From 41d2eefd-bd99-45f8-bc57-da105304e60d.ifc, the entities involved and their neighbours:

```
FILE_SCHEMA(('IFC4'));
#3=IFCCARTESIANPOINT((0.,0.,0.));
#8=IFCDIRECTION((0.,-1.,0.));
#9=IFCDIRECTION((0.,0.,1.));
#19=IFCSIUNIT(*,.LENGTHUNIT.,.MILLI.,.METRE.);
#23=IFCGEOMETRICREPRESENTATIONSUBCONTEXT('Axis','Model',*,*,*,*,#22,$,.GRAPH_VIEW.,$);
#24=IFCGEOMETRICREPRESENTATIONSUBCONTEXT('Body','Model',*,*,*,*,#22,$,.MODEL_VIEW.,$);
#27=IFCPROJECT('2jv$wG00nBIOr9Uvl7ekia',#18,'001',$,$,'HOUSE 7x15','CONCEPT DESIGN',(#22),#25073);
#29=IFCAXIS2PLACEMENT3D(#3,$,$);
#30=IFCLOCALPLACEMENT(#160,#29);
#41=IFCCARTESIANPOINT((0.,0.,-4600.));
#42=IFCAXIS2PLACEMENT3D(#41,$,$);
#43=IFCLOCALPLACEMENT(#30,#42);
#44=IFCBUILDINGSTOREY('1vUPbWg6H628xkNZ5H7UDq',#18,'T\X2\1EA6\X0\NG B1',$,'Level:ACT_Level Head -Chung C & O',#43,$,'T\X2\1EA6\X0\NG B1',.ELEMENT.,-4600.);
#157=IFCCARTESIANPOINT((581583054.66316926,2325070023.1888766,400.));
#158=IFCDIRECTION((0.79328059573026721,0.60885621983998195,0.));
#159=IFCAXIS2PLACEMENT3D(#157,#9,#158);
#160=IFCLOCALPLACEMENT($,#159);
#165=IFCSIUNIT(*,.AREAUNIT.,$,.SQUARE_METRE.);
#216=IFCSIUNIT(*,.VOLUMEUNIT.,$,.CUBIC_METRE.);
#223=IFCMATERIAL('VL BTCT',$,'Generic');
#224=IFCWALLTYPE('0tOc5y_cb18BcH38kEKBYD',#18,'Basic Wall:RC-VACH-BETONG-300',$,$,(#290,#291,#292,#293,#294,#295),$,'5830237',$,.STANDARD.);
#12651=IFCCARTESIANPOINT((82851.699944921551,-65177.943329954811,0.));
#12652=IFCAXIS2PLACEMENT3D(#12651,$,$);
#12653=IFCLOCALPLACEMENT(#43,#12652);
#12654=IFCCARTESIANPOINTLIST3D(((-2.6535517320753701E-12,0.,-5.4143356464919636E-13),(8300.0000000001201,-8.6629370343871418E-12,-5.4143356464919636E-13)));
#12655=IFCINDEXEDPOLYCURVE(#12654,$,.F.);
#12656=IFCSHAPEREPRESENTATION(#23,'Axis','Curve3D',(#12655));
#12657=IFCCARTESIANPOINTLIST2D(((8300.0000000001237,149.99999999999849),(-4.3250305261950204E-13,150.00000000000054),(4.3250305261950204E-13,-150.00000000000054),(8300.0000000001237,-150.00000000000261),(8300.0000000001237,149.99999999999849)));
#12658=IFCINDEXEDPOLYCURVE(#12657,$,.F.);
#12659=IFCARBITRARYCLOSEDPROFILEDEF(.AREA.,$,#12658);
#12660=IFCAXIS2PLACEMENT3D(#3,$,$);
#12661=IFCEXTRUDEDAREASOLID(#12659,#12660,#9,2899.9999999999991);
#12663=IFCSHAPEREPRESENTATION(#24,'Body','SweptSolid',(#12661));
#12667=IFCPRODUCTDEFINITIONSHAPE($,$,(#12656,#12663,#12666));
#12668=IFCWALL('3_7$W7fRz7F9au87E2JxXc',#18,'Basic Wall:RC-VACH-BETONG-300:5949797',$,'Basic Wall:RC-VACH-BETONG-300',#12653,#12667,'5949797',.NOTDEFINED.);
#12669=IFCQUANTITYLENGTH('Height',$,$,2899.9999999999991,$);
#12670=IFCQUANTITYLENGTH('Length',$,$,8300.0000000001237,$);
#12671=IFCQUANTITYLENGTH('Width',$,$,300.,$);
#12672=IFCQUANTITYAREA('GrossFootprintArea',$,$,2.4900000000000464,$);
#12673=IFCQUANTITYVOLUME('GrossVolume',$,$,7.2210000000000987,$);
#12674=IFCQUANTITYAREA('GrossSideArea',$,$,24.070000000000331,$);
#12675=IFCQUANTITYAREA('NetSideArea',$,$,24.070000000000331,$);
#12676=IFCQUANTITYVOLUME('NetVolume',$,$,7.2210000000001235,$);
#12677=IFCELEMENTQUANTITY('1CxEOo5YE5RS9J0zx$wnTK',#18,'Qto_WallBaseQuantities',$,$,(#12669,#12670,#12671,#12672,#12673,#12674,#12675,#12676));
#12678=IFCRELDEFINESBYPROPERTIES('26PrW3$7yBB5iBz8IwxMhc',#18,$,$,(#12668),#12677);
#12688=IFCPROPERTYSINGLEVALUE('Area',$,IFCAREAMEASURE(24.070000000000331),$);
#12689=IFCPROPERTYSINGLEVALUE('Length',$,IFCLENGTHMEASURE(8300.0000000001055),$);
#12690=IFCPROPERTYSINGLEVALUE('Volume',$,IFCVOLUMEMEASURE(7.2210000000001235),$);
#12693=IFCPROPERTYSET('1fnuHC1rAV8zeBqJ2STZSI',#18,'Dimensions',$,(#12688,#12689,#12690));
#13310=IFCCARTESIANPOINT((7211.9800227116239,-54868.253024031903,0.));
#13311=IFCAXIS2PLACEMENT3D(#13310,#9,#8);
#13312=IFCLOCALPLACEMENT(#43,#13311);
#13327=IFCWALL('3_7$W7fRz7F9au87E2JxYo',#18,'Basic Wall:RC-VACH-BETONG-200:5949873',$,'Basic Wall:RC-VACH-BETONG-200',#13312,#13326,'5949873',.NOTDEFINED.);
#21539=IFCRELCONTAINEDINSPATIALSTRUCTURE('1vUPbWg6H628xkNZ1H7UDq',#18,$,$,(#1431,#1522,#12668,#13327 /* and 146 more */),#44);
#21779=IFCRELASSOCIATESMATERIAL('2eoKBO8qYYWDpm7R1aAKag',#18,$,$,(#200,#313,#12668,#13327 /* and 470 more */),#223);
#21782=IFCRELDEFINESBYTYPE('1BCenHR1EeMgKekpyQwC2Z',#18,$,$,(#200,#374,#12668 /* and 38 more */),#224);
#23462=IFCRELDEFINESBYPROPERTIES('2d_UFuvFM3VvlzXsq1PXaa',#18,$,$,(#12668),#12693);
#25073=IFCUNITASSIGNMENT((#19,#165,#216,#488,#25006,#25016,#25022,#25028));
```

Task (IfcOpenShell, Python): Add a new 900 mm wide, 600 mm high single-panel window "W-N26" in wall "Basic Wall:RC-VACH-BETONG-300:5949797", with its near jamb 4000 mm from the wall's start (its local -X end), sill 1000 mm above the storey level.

```python
import numpy as np
import ifcopenshell
import ifcopenshell.api.feature
import ifcopenshell.api.geometry
import ifcopenshell.api.pset
import ifcopenshell.api.root
import ifcopenshell.api.spatial
import ifcopenshell.geom
import ifcopenshell.util.element
import ifcopenshell.util.placement
import ifcopenshell.util.representation
import ifcopenshell.util.shape
import ifcopenshell.util.unit

model = ifcopenshell.open("41d2eefd-bd99-45f8-bc57-da105304e60d.ifc")
unit_scale = ifcopenshell.util.unit.calculate_unit_scale(model)
area_scale = ifcopenshell.util.unit.calculate_unit_scale(model, "AREAUNIT")
volume_scale = ifcopenshell.util.unit.calculate_unit_scale(model, "VOLUMEUNIT")
settings = ifcopenshell.geom.settings()


def volume(element):
    """Net volume in cubic metres, openings subtracted."""
    shape = ifcopenshell.geom.create_shape(settings, element)
    return ifcopenshell.util.shape.get_volume(shape.geometry)


wall = model.by_guid("3_7$W7fRz7F9au87E2JxXc")
storey = ifcopenshell.util.element.get_container(wall, ifc_class="IfcBuildingStorey")
context = ifcopenshell.util.representation.get_context(model, "Model", "Body", "MODEL_VIEW")
before = volume(wall)

width, height, from_end, sill = 0.9, 0.6, 4, 1  # metres

# The wall runs along its own X axis, and the end named is its -X end.
wall_shape = ifcopenshell.geom.create_shape(settings, wall)
x, y, z = ifcopenshell.util.shape.get_vertices(wall_shape.geometry).T
start = x.min() + from_end
face, thickness = float(y.min()), float(y.max() - y.min())
wall_matrix = ifcopenshell.util.placement.get_local_placement(wall.ObjectPlacement)
level = ifcopenshell.util.placement.get_local_placement(storey.ObjectPlacement)[2, 3]


def in_wall(x, y):
    """Placement at x, y metres in the wall's axes, at sill height."""
    matrix = wall_matrix.copy()
    matrix[:, 3] = wall_matrix @ np.array([x / unit_scale, y / unit_scale, 0.0, 1.0])
    matrix[2, 3] = level + sill / unit_scale
    return matrix


# Opening: a box that overshoots both wall faces by 50 mm.
opening = ifcopenshell.api.root.create_entity(model, ifc_class="IfcOpeningElement", predefined_type="OPENING")
box = ifcopenshell.api.geometry.add_wall_representation(
    model, context=context, length=width, height=height, thickness=thickness + 0.1
)
ifcopenshell.api.geometry.assign_representation(model, product=opening, representation=box)
ifcopenshell.api.geometry.edit_object_placement(model, product=opening, matrix=in_wall(start, face - 0.05), is_si=False)
ifcopenshell.api.feature.add_feature(model, feature=opening, element=wall)

window = ifcopenshell.api.root.create_entity(model, ifc_class="IfcWindow", name="W-N26", predefined_type="WINDOW")
window.OverallWidth, window.OverallHeight = width / unit_scale, height / unit_scale
window.PartitioningType = "SINGLE_PANEL"
body = ifcopenshell.api.geometry.add_window_representation(
    model,
    context=context,
    overall_width=window.OverallWidth,
    overall_height=window.OverallHeight,
    partition_type="SINGLE_PANEL",
)
ifcopenshell.api.geometry.assign_representation(model, product=window, representation=body)
ifcopenshell.api.spatial.assign_container(model, products=[window], relating_structure=storey)
ifcopenshell.api.feature.add_filling(model, opening=opening, element=window)

# Centre the window in the wall's thickness.
ifcopenshell.api.geometry.edit_object_placement(model, product=window, matrix=in_wall(start, face), is_si=False)
window_shape = ifcopenshell.geom.create_shape(settings, window)
depth = ifcopenshell.util.shape.get_vertices(window_shape.geometry)[:, 1]
offset = face + thickness / 2 - (depth.min() + depth.max()) / 2
ifcopenshell.api.geometry.edit_object_placement(model, product=window, matrix=in_wall(start, offset), is_si=False)

after = volume(wall)

# Update the wall's stored quantities.
qto = model.by_id(ifcopenshell.util.element.get_pset(wall, "Qto_WallBaseQuantities", should_inherit=False)["id"])
ifcopenshell.api.pset.edit_qto(model, qto=qto, properties={
    "NetSideArea": after / thickness / area_scale,
    "NetVolume": after / volume_scale,
})
pset = model.by_id(ifcopenshell.util.element.get_pset(wall, "Dimensions", should_inherit=False)["id"])
ifcopenshell.api.pset.edit_pset(model, pset=pset, properties={
    "Area": model.create_entity("IfcAreaMeasure", after / thickness / area_scale),
    "Volume": model.create_entity("IfcVolumeMeasure", after / volume_scale),
})

print(f"wall volume {before:.3f} -> {after:.3f} m3")

model.write("41d2eefd-bd99-45f8-bc57-da105304e60d_edited.ifc")
```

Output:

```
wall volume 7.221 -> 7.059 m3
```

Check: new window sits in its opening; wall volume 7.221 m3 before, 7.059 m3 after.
